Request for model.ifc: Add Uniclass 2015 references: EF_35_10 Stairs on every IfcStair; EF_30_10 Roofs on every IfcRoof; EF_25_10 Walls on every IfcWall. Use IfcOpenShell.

First a look at what the model holds.

```python
import ifcopenshell

model = ifcopenshell.open("model.ifc")
print(model.schema)
print("classifications:", [c.Name for c in model.by_type("IfcClassification")])
for ifc_class in ("IfcDoor", "IfcRoof", "IfcStair", "IfcWall", "IfcWindow"):
    print(ifc_class, len(model.by_type(ifc_class)))
```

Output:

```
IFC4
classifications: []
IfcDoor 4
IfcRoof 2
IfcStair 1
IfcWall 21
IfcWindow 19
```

```python
import ifcopenshell
import ifcopenshell.api.classification

model = ifcopenshell.open("model.ifc")

system = ifcopenshell.api.classification.add_classification(model, classification="Uniclass 2015")

codes = {
    "IfcStair": ("EF_35_10", "Stairs"),
    "IfcRoof": ("EF_30_10", "Roofs"),
    "IfcWall": ("EF_25_10", "Walls"),
}
for ifc_class, (code, name) in codes.items():
    products = model.by_type(ifc_class)
    ifcopenshell.api.classification.add_reference(
        model, products=products, classification=system, identification=code, name=name
    )
    print(code, len(products))

model.write("model-out.ifc")
```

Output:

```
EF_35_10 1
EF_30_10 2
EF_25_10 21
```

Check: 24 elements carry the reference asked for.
